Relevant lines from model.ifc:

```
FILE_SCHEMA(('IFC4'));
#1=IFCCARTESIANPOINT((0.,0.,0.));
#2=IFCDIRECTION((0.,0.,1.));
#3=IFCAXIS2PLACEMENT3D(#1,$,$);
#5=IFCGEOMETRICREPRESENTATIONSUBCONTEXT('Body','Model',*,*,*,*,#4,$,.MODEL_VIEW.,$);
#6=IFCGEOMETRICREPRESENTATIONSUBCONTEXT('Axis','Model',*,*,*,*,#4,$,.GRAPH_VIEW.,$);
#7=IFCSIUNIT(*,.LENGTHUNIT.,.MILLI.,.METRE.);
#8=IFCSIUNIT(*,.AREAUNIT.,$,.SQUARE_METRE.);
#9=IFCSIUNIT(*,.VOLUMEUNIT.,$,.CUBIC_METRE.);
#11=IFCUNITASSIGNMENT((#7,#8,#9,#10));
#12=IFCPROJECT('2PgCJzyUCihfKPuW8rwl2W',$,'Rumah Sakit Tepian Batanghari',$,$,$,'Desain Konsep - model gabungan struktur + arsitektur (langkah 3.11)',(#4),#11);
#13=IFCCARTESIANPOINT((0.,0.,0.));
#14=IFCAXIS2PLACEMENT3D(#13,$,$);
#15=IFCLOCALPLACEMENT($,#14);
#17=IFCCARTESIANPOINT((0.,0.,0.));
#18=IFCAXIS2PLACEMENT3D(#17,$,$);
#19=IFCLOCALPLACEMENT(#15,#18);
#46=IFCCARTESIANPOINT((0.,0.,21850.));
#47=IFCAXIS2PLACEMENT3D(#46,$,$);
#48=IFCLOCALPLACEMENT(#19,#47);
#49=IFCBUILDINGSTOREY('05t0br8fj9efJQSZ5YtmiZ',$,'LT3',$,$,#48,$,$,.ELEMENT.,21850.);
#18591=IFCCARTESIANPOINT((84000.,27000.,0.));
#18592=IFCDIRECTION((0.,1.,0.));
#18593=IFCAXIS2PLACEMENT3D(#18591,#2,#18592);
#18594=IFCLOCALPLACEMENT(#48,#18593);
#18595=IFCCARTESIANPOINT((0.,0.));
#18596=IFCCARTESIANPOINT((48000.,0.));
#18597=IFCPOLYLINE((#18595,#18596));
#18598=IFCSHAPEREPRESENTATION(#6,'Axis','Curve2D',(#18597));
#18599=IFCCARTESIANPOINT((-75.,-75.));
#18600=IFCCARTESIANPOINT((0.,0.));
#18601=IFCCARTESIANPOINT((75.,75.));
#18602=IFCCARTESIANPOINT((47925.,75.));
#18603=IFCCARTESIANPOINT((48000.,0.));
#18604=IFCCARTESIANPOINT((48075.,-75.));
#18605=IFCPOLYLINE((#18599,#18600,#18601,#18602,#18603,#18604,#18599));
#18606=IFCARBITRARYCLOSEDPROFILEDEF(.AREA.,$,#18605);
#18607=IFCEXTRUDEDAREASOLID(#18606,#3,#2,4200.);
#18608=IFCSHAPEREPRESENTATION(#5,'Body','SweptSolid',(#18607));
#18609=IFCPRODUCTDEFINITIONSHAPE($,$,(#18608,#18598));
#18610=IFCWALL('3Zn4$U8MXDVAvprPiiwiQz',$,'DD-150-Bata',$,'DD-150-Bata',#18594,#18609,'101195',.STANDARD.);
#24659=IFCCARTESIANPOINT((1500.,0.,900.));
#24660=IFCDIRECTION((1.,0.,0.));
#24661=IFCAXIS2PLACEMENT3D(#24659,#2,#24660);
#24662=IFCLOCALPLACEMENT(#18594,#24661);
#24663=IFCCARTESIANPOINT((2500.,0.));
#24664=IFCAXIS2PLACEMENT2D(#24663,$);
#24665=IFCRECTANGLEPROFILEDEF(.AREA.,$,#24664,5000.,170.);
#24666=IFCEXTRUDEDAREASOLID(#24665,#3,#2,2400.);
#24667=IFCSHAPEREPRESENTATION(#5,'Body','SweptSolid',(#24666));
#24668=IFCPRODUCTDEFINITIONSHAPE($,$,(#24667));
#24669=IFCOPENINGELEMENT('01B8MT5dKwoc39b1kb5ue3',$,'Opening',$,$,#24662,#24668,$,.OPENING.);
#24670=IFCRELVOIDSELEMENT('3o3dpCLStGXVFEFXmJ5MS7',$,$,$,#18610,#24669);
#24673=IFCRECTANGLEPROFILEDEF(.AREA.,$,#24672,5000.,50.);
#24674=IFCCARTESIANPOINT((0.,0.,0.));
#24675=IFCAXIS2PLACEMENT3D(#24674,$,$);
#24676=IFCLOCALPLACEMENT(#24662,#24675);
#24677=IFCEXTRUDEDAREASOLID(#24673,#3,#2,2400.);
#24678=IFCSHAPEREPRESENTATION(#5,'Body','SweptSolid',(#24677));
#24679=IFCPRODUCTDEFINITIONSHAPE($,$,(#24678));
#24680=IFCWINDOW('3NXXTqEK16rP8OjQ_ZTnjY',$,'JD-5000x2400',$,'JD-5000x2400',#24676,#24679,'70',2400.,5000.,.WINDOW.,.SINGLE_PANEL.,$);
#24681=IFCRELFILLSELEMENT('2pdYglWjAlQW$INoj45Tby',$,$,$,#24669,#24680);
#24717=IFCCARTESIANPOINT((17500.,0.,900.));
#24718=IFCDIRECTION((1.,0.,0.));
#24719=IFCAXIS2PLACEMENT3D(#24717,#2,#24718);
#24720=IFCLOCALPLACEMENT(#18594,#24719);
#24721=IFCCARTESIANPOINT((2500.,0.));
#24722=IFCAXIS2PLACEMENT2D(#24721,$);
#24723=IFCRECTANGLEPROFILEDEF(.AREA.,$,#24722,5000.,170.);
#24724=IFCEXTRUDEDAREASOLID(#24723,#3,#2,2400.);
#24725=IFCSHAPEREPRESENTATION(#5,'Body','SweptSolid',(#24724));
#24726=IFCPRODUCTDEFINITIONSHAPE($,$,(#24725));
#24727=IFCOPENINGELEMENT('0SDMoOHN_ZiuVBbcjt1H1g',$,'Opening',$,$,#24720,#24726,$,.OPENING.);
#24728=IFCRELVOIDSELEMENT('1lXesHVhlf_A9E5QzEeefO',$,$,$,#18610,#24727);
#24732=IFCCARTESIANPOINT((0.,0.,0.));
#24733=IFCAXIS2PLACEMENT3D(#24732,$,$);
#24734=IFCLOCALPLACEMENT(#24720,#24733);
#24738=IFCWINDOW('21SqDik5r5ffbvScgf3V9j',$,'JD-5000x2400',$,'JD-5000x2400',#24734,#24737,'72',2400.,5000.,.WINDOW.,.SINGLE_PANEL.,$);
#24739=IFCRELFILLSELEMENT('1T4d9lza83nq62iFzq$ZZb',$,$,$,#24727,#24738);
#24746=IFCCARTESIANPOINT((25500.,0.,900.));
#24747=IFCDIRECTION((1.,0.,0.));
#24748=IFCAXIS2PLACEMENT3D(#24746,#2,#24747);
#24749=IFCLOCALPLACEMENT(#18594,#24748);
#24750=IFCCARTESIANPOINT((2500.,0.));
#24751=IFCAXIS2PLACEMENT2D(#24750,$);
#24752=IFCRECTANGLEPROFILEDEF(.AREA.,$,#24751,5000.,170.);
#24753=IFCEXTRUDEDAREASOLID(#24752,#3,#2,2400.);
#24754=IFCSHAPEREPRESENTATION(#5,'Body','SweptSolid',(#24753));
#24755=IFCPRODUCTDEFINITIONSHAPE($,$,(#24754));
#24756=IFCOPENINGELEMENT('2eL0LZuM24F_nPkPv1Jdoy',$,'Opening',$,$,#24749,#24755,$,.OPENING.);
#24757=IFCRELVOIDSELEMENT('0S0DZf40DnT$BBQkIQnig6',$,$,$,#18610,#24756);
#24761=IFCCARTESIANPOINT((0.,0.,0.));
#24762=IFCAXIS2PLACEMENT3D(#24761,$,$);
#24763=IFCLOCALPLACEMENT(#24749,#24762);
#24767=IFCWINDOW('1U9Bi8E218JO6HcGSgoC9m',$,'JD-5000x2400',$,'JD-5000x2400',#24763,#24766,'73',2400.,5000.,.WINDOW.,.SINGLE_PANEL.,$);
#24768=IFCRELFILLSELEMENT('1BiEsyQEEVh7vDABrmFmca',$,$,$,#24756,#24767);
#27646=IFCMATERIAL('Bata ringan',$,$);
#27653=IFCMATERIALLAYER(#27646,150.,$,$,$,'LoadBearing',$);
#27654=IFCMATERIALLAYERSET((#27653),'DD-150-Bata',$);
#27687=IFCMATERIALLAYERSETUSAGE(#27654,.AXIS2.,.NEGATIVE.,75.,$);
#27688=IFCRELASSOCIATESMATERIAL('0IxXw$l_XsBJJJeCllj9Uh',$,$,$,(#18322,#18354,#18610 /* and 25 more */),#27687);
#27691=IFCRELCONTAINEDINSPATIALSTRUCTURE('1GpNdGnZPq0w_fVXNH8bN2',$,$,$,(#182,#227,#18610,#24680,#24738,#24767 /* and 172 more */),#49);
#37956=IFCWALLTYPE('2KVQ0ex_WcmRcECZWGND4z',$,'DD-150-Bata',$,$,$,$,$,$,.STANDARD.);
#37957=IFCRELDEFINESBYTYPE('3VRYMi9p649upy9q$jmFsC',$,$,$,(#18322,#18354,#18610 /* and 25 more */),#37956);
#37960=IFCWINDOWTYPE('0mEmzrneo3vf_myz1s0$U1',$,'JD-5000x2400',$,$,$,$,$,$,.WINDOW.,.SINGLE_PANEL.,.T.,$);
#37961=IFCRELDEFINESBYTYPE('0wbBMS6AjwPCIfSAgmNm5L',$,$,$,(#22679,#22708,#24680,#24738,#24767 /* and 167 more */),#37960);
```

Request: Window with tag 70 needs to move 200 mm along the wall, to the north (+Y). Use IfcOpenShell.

```python
import ifcopenshell
import ifcopenshell.api.geometry
import ifcopenshell.util.placement

model = ifcopenshell.open("model.ifc")

window = model.by_id(24680)
opening = window.FillsVoids[0].RelatingOpeningElement
wall = opening.VoidsElements[0].RelatingBuildingElement

wall_matrix = ifcopenshell.util.placement.get_local_placement(wall.ObjectPlacement)
shift = wall_matrix[:3, 0] * 200.0
before = ifcopenshell.util.placement.get_local_placement(window.ObjectPlacement)[:3, 3].copy()

# The window is placed relative to its opening, so it follows when the opening moves.
matrix = ifcopenshell.util.placement.get_local_placement(opening.ObjectPlacement)
matrix[:3, 3] += shift
ifcopenshell.api.geometry.edit_object_placement(
    model, product=opening, matrix=matrix, is_si=False, should_transform_children=True
)

after = ifcopenshell.util.placement.get_local_placement(window.ObjectPlacement)[:3, 3]
print("window moved by", (after - before).round(3) + 0.0)

model.write("model_rev.ifc")
```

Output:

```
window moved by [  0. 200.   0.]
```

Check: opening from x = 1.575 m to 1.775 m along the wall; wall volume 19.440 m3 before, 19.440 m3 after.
